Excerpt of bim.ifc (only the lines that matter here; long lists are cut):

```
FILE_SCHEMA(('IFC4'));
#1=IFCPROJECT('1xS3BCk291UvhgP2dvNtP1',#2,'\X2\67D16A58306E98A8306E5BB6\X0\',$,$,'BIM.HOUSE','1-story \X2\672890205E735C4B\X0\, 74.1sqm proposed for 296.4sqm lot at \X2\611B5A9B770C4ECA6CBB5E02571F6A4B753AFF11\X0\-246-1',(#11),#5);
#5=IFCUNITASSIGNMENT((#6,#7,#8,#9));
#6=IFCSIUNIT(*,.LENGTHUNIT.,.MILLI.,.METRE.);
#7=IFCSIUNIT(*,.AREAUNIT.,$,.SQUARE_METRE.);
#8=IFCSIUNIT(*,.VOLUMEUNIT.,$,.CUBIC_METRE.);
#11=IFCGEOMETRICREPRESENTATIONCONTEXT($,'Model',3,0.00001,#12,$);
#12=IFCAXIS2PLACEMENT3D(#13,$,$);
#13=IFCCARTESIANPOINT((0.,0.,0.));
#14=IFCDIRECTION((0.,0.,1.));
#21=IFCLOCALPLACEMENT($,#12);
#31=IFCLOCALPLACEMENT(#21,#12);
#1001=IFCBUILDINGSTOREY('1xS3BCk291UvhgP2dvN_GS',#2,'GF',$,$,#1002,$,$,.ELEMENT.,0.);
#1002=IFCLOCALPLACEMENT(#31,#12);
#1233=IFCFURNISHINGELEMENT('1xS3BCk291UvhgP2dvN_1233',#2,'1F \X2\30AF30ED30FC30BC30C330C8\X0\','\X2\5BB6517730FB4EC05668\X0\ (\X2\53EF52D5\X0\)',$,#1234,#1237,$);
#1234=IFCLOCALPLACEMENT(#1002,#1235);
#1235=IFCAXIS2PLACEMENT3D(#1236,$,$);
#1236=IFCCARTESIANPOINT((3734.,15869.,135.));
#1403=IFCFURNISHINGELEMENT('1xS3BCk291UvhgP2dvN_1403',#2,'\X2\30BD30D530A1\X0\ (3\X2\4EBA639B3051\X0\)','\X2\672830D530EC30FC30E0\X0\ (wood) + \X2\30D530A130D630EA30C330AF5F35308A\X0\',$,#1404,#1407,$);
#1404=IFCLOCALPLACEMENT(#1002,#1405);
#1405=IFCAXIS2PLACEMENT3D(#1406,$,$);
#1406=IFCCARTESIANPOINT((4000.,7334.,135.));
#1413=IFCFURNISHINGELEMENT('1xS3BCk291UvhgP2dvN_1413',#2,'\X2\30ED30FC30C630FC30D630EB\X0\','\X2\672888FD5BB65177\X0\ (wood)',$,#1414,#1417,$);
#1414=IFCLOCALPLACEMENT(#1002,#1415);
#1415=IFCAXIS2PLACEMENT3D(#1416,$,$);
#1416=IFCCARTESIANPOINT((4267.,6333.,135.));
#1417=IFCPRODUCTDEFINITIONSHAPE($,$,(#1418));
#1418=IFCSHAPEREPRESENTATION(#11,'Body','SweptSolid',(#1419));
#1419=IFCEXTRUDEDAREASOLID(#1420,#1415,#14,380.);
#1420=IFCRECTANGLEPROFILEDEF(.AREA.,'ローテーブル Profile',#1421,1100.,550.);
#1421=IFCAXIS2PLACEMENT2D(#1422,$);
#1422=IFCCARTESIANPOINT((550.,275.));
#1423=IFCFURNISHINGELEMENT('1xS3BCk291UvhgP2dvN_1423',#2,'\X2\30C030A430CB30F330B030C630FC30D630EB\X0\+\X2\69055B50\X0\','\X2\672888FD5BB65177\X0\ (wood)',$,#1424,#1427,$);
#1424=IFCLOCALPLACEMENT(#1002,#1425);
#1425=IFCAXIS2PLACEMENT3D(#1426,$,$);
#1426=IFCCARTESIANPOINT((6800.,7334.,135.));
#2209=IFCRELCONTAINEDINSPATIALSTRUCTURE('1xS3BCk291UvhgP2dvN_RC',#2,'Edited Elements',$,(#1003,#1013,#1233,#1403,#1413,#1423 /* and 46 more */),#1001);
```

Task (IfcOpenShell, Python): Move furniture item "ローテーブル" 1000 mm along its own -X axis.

```python
import ifcopenshell
import ifcopenshell.api.geometry
import ifcopenshell.util.placement

model = ifcopenshell.open("bim.ifc")

item = model.by_guid("1xS3BCk291UvhgP2dvN_1413")
matrix = ifcopenshell.util.placement.get_local_placement(item.ObjectPlacement)
matrix[:3, 3] -= matrix[:3, 0] * 1000.0
ifcopenshell.api.geometry.edit_object_placement(model, product=item, matrix=matrix, is_si=False)

print(ifcopenshell.util.placement.get_local_placement(item.ObjectPlacement).round(3) + 0.0)

model.write("bim-out.ifc")
```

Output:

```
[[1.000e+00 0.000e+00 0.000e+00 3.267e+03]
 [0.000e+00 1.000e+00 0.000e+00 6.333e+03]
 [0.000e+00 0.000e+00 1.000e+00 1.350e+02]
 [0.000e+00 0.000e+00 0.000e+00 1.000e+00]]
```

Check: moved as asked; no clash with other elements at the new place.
